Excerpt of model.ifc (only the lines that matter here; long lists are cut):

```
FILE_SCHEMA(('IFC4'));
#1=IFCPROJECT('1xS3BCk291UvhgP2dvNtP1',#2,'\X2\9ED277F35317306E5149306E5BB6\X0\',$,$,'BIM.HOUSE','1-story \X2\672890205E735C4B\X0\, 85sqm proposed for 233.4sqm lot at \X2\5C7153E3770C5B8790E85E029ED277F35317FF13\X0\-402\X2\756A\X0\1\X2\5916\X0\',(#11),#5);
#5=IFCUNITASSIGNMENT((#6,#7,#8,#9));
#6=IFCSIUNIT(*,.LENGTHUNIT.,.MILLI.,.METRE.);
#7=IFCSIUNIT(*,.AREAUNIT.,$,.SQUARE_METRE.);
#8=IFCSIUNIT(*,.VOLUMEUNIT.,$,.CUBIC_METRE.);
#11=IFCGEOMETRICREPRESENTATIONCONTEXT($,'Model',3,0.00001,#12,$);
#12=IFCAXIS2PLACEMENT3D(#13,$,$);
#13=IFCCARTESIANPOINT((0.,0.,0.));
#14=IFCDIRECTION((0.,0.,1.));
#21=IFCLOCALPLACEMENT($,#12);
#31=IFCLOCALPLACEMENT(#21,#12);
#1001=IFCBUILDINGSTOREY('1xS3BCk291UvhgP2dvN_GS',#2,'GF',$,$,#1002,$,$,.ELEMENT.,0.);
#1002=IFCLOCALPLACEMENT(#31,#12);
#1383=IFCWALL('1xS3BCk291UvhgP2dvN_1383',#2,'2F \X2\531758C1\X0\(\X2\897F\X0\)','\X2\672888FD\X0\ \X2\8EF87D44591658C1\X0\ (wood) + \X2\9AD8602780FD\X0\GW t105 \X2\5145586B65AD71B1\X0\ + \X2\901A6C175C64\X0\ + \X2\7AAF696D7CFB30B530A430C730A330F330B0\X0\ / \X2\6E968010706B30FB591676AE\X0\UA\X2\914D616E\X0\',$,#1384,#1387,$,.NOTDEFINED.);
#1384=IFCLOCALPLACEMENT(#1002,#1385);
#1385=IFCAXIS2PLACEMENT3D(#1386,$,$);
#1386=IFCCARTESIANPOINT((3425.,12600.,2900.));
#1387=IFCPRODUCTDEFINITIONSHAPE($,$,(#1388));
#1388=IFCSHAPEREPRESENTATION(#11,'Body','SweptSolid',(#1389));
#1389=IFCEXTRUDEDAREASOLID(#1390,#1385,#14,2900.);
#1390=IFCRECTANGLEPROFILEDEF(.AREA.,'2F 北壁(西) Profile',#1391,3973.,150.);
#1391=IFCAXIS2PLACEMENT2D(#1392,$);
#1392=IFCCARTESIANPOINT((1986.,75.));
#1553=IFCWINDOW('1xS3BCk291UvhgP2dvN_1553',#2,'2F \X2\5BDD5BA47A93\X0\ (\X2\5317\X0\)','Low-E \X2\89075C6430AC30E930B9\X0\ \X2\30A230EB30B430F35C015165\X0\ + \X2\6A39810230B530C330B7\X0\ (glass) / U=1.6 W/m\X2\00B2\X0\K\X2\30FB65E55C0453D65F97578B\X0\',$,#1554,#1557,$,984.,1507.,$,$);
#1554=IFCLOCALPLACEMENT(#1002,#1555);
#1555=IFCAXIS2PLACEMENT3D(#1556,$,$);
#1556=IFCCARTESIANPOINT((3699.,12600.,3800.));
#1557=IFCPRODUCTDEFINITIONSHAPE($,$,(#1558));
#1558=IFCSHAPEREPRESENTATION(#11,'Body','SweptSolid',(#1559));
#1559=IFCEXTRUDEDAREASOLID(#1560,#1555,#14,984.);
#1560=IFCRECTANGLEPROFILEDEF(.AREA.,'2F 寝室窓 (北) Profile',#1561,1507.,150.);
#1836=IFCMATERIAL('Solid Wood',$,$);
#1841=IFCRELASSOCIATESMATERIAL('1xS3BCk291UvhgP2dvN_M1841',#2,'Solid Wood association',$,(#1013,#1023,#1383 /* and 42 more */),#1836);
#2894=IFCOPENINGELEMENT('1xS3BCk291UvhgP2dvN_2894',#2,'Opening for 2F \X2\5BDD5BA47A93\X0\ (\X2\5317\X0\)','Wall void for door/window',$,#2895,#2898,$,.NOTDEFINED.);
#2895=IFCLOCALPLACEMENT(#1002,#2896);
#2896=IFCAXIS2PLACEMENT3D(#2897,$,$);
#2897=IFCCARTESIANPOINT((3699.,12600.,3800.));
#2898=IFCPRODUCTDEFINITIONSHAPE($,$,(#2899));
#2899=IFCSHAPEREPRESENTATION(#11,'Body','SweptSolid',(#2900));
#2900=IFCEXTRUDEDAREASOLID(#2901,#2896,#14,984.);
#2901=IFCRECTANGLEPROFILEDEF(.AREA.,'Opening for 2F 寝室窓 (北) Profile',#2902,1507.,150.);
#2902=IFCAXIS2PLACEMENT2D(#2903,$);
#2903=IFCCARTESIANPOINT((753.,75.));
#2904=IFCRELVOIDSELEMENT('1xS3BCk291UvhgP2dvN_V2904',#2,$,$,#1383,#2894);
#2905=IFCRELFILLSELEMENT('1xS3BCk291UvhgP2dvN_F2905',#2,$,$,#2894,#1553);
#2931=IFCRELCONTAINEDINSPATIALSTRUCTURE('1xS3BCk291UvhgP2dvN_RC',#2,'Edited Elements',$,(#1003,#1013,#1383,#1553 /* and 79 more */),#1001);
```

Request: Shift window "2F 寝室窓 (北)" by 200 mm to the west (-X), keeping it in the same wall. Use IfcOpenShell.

```python
import ifcopenshell
import ifcopenshell.api.geometry
import ifcopenshell.util.placement

model = ifcopenshell.open("model.ifc")

window = model.by_id(1553)
opening = window.FillsVoids[0].RelatingOpeningElement
wall = opening.VoidsElements[0].RelatingBuildingElement

wall_matrix = ifcopenshell.util.placement.get_local_placement(wall.ObjectPlacement)
shift = wall_matrix[:3, 0] * -200.0
before = ifcopenshell.util.placement.get_local_placement(window.ObjectPlacement)[:3, 3].copy()

# The window is not placed relative to its opening, so move both.
for product in (opening, window):
    matrix = ifcopenshell.util.placement.get_local_placement(product.ObjectPlacement)
    matrix[:3, 3] += shift
    ifcopenshell.api.geometry.edit_object_placement(model, product=product, matrix=matrix, is_si=False)

after = ifcopenshell.util.placement.get_local_placement(window.ObjectPlacement)[:3, 3]
print("window moved by", (after - before).round(3) + 0.0)

model.write("model-out.ifc")
```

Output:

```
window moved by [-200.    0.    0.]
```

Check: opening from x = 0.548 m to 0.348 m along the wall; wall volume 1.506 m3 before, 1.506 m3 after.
